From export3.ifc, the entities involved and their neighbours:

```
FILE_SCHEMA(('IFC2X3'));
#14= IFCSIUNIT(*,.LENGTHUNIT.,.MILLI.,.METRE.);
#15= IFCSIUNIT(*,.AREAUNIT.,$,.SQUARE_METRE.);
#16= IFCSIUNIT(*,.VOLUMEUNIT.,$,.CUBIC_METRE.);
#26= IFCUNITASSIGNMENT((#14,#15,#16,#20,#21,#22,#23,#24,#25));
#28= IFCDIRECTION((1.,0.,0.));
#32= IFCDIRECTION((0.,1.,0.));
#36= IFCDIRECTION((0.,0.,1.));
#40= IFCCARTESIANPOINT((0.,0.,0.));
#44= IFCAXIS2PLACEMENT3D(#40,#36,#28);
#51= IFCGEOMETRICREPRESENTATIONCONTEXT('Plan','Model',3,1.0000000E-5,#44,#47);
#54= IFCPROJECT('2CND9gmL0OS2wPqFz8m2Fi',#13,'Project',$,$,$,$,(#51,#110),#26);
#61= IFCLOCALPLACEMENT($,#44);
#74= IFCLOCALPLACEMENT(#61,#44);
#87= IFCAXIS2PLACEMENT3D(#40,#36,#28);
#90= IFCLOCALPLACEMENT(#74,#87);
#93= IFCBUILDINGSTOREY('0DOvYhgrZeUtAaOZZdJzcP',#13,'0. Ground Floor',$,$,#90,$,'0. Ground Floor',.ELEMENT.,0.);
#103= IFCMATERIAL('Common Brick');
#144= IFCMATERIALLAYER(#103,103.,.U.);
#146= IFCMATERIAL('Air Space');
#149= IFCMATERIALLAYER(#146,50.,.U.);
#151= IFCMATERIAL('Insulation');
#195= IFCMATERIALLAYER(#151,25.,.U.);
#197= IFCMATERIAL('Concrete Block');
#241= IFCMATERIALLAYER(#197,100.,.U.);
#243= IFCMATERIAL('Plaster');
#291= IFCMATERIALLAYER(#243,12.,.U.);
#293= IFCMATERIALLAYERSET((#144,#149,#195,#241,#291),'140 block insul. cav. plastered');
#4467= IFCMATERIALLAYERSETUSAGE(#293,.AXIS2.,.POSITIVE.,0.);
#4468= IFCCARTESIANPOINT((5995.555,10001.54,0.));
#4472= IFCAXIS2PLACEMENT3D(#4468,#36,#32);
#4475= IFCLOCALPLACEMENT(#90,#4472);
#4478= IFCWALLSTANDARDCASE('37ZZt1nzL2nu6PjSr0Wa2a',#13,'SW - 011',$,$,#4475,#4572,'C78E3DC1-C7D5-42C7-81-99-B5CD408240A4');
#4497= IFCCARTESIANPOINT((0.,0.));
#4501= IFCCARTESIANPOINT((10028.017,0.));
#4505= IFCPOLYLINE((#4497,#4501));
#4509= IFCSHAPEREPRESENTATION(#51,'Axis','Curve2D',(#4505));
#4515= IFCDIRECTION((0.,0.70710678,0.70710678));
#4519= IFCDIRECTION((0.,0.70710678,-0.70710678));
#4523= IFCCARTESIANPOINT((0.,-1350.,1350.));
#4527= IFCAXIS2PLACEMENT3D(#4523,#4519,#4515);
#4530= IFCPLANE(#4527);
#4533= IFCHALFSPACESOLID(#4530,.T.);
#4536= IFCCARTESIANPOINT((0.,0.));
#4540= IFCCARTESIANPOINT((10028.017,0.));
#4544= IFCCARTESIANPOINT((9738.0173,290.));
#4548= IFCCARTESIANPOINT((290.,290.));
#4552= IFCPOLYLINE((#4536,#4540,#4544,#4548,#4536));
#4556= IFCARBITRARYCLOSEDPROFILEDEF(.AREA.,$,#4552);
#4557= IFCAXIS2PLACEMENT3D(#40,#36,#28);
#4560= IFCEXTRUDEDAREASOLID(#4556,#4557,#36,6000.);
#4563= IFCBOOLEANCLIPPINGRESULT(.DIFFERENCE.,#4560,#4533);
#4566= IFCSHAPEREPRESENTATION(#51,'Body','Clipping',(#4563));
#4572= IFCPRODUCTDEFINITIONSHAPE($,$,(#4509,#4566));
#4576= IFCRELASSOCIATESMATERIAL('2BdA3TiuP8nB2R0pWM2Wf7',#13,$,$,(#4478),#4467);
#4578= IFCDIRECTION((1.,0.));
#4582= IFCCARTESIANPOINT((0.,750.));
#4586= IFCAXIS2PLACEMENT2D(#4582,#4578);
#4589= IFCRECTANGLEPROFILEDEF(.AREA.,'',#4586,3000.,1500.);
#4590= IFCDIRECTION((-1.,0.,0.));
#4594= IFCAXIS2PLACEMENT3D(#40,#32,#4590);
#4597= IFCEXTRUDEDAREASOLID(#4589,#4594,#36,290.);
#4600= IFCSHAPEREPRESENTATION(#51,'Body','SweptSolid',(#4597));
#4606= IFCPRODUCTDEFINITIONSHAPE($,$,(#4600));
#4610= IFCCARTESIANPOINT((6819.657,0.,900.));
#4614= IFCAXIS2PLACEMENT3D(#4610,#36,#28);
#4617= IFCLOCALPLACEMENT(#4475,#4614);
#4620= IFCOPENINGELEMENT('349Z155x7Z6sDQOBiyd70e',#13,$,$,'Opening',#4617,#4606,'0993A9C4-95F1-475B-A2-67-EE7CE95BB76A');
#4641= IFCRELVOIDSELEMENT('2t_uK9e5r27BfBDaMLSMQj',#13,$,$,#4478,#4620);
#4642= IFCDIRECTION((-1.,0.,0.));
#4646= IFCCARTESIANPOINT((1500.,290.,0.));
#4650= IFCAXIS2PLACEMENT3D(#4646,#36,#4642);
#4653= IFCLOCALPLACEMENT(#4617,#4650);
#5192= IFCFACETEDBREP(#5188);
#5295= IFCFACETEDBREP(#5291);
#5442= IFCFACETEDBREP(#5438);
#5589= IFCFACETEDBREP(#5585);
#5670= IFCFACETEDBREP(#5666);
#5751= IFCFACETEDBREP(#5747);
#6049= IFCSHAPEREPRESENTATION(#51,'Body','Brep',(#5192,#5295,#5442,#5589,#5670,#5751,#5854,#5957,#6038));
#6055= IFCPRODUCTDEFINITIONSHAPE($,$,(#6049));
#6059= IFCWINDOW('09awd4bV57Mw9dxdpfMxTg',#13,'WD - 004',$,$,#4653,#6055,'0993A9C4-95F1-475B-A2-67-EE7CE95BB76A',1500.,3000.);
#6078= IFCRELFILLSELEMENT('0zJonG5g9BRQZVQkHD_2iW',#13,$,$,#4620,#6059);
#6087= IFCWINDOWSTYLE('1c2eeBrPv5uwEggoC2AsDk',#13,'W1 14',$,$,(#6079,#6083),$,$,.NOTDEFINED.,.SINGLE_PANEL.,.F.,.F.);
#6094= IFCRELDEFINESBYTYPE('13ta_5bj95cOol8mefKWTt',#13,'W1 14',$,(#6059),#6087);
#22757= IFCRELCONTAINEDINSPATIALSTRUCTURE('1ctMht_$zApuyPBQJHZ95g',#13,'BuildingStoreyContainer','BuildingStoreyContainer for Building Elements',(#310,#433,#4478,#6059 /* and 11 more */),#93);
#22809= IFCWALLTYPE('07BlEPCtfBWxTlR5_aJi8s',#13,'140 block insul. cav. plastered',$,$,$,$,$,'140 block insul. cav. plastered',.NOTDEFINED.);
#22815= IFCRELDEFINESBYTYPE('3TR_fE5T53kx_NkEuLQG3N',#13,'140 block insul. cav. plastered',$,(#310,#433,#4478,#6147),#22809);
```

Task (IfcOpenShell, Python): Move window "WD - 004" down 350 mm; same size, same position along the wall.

```python
import numpy as np
import ifcopenshell
import ifcopenshell.api.geometry
import ifcopenshell.util.placement
import ifcopenshell.util.unit

model = ifcopenshell.open("export3.ifc")
unit_scale = ifcopenshell.util.unit.calculate_unit_scale(model)

window = model.by_guid("09awd4bV57Mw9dxdpfMxTg")
opening = window.FillsVoids[0].RelatingOpeningElement
dz = -350.0

shift = np.array([0.0, 0.0, dz])
# The window is placed relative to its opening, so it follows when the opening moves.
matrix = ifcopenshell.util.placement.get_local_placement(opening.ObjectPlacement)
matrix[:3, 3] += shift
ifcopenshell.api.geometry.edit_object_placement(
    model, product=opening, matrix=matrix, is_si=False, should_transform_children=True
)

print(f"moved by {dz * unit_scale:+.3f} m")

model.write("export3_updated.ifc")
```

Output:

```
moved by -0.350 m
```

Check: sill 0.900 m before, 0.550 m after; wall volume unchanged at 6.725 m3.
